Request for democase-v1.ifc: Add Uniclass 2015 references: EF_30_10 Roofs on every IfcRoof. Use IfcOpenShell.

First a look at what the model holds.

```python
import ifcopenshell

model = ifcopenshell.open("democase-v1.ifc")
print(model.schema)
print("classifications:", [c.Name for c in model.by_type("IfcClassification")])
for ifc_class in ("IfcDoor", "IfcRoof", "IfcStair", "IfcWall", "IfcWindow"):
    print(ifc_class, len(model.by_type(ifc_class)))
```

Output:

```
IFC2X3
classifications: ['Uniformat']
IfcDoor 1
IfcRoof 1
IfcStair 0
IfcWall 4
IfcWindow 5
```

```python
import ifcopenshell
import ifcopenshell.api.classification

model = ifcopenshell.open("democase-v1.ifc")

# IFC2X3 requires Source and Edition and has no link from the project to the system.
system = model.create_entity("IfcClassification", Source="NBS", Edition="2015", Name="Uniclass 2015")

codes = {
    "IfcRoof": ("EF_30_10", "Roofs"),
}
for ifc_class, (code, name) in codes.items():
    products = model.by_type(ifc_class)
    ifcopenshell.api.classification.add_reference(
        model, products=products, classification=system, identification=code, name=name
    )
    print(code, len(products))

model.write("democase-v1_rev.ifc")
```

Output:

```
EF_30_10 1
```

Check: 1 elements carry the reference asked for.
